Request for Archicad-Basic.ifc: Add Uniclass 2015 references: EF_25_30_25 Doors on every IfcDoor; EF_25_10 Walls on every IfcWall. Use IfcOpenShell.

First a look at what the model holds.

```python
import ifcopenshell

model = ifcopenshell.open("Archicad-Basic.ifc")
print(model.schema)
print("classifications:", [c.Name for c in model.by_type("IfcClassification")])
for ifc_class in ("IfcDoor", "IfcRoof", "IfcStair", "IfcWall", "IfcWindow"):
    print(ifc_class, len(model.by_type(ifc_class)))
```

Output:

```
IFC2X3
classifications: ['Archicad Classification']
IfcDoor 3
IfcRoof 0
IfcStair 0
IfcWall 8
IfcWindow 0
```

```python
import ifcopenshell
import ifcopenshell.api.classification

model = ifcopenshell.open("Archicad-Basic.ifc")

# IFC2X3 requires Source and Edition and has no link from the project to the system.
system = model.create_entity("IfcClassification", Source="NBS", Edition="2015", Name="Uniclass 2015")

codes = {
    "IfcDoor": ("EF_25_30_25", "Doors"),
    "IfcWall": ("EF_25_10", "Walls"),
}
for ifc_class, (code, name) in codes.items():
    products = model.by_type(ifc_class)
    ifcopenshell.api.classification.add_reference(
        model, products=products, classification=system, identification=code, name=name
    )
    print(code, len(products))

model.write("Archicad-Basic_edited.ifc")
```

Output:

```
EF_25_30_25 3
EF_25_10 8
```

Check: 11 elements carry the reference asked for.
